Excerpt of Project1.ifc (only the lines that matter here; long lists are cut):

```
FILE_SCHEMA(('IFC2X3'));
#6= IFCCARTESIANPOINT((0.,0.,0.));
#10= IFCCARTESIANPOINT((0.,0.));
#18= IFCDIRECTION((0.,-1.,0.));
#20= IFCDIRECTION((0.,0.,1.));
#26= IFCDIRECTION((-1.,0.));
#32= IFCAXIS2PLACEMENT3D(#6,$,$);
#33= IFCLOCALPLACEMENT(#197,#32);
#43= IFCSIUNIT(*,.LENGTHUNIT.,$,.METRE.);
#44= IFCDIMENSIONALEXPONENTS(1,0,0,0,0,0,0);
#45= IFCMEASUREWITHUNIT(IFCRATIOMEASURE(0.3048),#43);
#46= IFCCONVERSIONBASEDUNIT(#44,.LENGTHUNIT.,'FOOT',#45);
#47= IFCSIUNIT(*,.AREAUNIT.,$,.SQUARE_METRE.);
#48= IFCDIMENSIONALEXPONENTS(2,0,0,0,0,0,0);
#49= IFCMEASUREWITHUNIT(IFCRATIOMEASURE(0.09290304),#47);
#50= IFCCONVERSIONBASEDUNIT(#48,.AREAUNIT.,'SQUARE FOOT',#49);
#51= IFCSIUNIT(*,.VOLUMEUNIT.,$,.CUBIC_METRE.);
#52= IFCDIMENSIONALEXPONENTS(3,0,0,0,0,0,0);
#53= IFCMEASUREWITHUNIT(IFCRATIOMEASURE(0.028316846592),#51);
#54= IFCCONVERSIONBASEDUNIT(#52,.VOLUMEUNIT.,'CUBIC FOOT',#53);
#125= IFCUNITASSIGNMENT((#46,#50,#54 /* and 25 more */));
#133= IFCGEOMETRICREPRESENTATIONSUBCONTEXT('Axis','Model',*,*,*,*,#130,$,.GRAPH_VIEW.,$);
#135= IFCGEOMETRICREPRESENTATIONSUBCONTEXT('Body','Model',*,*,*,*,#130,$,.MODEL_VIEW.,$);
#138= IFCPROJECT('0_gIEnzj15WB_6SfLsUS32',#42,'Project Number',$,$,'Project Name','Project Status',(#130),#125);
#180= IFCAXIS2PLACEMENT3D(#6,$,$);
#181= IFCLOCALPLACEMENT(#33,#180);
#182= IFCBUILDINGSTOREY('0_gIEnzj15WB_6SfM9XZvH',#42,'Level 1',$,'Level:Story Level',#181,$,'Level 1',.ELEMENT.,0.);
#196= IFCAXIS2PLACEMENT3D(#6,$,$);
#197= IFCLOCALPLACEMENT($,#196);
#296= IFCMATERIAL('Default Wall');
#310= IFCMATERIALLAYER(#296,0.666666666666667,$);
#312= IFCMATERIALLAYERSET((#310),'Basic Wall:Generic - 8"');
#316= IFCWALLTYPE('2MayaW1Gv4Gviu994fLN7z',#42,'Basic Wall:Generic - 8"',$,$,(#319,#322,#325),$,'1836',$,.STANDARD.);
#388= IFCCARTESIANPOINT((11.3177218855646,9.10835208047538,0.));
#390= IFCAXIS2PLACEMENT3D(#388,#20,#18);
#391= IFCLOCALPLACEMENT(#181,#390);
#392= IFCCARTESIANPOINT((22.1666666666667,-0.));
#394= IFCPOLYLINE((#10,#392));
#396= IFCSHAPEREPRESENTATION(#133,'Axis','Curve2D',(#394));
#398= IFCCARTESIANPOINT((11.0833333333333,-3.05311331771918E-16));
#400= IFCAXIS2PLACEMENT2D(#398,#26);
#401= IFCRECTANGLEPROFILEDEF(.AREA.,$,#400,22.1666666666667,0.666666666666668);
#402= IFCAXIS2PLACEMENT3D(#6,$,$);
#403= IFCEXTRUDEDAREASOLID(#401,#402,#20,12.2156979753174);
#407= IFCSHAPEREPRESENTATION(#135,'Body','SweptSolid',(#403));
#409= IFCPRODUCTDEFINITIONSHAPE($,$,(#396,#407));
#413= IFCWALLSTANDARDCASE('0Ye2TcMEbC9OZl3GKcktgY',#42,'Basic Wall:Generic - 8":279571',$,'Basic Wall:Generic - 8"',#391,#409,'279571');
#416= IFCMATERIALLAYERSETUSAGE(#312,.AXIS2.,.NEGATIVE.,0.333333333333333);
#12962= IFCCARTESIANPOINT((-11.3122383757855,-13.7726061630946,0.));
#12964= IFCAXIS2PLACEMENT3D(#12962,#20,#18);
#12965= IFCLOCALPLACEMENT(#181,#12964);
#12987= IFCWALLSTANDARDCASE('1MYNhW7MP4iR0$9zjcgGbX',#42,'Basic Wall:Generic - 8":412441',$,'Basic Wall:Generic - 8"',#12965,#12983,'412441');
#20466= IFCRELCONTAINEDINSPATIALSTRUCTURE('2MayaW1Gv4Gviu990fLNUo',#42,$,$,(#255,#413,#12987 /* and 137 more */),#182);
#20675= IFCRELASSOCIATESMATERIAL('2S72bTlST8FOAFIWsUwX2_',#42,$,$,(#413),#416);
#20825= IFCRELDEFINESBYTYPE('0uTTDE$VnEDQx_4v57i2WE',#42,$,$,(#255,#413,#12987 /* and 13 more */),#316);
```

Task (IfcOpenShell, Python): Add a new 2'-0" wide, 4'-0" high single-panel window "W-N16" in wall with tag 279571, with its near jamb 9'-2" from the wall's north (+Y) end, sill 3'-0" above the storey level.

```python
import numpy as np
import ifcopenshell
import ifcopenshell.api.feature
import ifcopenshell.api.geometry
import ifcopenshell.api.root
import ifcopenshell.api.spatial
import ifcopenshell.api.type
import ifcopenshell.geom
import ifcopenshell.util.element
import ifcopenshell.util.placement
import ifcopenshell.util.representation
import ifcopenshell.util.shape
import ifcopenshell.util.unit

model = ifcopenshell.open("Project1.ifc")
unit_scale = ifcopenshell.util.unit.calculate_unit_scale(model)
settings = ifcopenshell.geom.settings()


def volume(element):
    """Net volume in cubic metres, openings subtracted."""
    shape = ifcopenshell.geom.create_shape(settings, element)
    return ifcopenshell.util.shape.get_volume(shape.geometry)


wall = model.by_guid("0Ye2TcMEbC9OZl3GKcktgY")
storey = ifcopenshell.util.element.get_container(wall, ifc_class="IfcBuildingStorey")
context = ifcopenshell.util.representation.get_context(model, "Model", "Body", "MODEL_VIEW")
before = volume(wall)

width, height, from_end, sill = 0.6096, 1.2192, 2.794, 0.9144  # metres

# The wall runs along its own X axis, and the end named is its -X end.
wall_shape = ifcopenshell.geom.create_shape(settings, wall)
x, y, z = ifcopenshell.util.shape.get_vertices(wall_shape.geometry).T
start = x.min() + from_end
face, thickness = float(y.min()), float(y.max() - y.min())
wall_matrix = ifcopenshell.util.placement.get_local_placement(wall.ObjectPlacement)
level = ifcopenshell.util.placement.get_local_placement(storey.ObjectPlacement)[2, 3]


def in_wall(x, y):
    """Placement at x, y metres in the wall's axes, at sill height."""
    matrix = wall_matrix.copy()
    matrix[:, 3] = wall_matrix @ np.array([x / unit_scale, y / unit_scale, 0.0, 1.0])
    matrix[2, 3] = level + sill / unit_scale
    return matrix


# Opening: a box that overshoots both wall faces by 50 mm.
opening = ifcopenshell.api.root.create_entity(model, ifc_class="IfcOpeningElement")
box = ifcopenshell.api.geometry.add_wall_representation(
    model, context=context, length=width, height=height, thickness=thickness + 0.1
)
ifcopenshell.api.geometry.assign_representation(model, product=opening, representation=box)
ifcopenshell.api.geometry.edit_object_placement(model, product=opening, matrix=in_wall(start, face - 0.05), is_si=False)
ifcopenshell.api.feature.add_feature(model, feature=opening, element=wall)

window = ifcopenshell.api.root.create_entity(model, ifc_class="IfcWindow", name="W-N16")
window.OverallWidth, window.OverallHeight = width / unit_scale, height / unit_scale
body = ifcopenshell.api.geometry.add_window_representation(
    model,
    context=context,
    overall_width=window.OverallWidth,
    overall_height=window.OverallHeight,
    partition_type="SINGLE_PANEL",
)
ifcopenshell.api.geometry.assign_representation(model, product=window, representation=body)
ifcopenshell.api.spatial.assign_container(model, products=[window], relating_structure=storey)
fills = ifcopenshell.api.feature.add_filling(model, opening=opening, element=window)
fills.OwnerHistory = window.OwnerHistory  # required in IFC2X3

# IFC2X3 keeps the operation on the window style.
style = ifcopenshell.api.root.create_entity(model, ifc_class="IfcWindowStyle", name="W-N16")
style.OperationType, style.ConstructionType = "SINGLE_PANEL", "NOTDEFINED"
style.ParameterTakesPrecedence = style.Sizeable = False
ifcopenshell.api.type.assign_type(model, related_objects=[window], relating_type=style)

# Centre the window in the wall's thickness.
ifcopenshell.api.geometry.edit_object_placement(model, product=window, matrix=in_wall(start, face), is_si=False)
window_shape = ifcopenshell.geom.create_shape(settings, window)
depth = ifcopenshell.util.shape.get_vertices(window_shape.geometry)[:, 1]
offset = face + thickness / 2 - (depth.min() + depth.max()) / 2
ifcopenshell.api.geometry.edit_object_placement(model, product=window, matrix=in_wall(start, offset), is_si=False)

after = volume(wall)

print(f"wall volume {before:.3f} -> {after:.3f} m3")

model.write("Project1_v2.ifc")
```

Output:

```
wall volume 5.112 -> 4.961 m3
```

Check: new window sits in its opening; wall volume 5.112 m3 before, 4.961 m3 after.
